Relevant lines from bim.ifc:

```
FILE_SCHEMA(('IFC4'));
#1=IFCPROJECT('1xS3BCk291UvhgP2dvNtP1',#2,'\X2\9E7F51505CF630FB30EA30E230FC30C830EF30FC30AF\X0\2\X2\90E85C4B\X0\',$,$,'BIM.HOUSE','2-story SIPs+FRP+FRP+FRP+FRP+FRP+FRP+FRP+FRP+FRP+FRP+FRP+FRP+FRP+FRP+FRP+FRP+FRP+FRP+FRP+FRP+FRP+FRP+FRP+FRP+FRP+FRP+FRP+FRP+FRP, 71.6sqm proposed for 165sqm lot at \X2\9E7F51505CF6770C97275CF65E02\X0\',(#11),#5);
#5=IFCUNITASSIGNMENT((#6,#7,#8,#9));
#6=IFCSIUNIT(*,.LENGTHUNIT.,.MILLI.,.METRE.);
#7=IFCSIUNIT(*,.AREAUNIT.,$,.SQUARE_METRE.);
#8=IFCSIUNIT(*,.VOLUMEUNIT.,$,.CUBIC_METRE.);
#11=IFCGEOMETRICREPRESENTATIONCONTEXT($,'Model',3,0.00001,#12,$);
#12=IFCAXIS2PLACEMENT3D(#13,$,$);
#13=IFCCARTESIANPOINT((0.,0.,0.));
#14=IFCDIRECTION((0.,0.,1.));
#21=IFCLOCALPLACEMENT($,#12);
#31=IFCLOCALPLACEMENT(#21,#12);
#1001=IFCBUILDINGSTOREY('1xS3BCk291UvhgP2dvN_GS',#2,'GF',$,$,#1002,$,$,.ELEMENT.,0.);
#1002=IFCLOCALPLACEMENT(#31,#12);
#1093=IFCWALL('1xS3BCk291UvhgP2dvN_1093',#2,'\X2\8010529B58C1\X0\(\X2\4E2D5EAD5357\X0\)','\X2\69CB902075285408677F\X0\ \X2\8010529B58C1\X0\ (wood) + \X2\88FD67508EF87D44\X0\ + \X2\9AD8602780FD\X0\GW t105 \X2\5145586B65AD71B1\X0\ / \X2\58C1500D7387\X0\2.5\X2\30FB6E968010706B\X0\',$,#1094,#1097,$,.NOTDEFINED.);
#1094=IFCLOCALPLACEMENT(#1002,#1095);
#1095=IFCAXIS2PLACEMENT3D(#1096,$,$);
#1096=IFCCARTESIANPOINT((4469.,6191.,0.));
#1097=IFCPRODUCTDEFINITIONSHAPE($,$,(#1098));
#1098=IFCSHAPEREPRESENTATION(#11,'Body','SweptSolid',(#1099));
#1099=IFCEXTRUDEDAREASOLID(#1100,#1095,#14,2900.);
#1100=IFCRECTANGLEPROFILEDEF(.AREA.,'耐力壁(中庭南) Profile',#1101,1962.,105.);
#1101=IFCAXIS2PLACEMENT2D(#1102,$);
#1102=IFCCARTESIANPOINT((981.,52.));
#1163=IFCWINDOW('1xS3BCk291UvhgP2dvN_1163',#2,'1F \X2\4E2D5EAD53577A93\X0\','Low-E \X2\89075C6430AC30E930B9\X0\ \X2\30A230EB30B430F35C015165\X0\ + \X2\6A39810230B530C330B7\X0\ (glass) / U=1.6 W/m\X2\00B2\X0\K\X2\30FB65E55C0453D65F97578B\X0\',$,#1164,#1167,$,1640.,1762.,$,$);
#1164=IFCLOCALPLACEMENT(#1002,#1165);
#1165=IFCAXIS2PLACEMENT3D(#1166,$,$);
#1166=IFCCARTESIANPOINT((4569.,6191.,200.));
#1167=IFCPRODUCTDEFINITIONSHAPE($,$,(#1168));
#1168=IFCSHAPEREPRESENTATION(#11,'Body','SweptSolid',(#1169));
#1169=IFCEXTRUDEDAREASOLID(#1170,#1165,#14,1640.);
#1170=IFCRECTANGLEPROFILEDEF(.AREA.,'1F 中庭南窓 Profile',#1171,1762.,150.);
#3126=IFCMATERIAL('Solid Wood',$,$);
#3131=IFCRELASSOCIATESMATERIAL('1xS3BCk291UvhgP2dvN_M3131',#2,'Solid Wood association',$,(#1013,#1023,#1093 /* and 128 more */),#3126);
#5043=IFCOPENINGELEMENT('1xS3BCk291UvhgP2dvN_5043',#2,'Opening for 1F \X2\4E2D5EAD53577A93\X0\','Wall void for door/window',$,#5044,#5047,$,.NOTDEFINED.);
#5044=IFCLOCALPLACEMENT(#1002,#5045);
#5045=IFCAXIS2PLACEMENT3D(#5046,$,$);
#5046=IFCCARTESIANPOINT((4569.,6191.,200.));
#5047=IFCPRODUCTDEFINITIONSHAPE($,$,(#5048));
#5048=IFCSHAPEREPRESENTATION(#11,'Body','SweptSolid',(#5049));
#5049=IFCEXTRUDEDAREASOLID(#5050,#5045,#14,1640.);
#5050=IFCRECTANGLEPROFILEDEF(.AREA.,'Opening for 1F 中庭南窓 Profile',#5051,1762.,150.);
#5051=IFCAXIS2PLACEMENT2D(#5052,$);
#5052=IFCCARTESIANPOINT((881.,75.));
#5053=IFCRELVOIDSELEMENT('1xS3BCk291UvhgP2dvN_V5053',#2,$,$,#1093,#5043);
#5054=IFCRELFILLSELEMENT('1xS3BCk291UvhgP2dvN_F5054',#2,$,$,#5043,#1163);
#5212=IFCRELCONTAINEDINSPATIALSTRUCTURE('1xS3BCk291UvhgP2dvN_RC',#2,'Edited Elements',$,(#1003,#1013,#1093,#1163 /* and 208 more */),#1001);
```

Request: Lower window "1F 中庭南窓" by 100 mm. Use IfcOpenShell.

```python
import numpy as np
import ifcopenshell
import ifcopenshell.api.geometry
import ifcopenshell.util.placement
import ifcopenshell.util.unit

model = ifcopenshell.open("bim.ifc")
unit_scale = ifcopenshell.util.unit.calculate_unit_scale(model)

window = model.by_guid("1xS3BCk291UvhgP2dvN_1163")
opening = window.FillsVoids[0].RelatingOpeningElement
dz = -100.0

shift = np.array([0.0, 0.0, dz])
# The window is not placed relative to its opening, so move both.
for product in (opening, window):
    matrix = ifcopenshell.util.placement.get_local_placement(product.ObjectPlacement)
    matrix[:3, 3] += shift
    ifcopenshell.api.geometry.edit_object_placement(model, product=product, matrix=matrix, is_si=False)

print(f"moved by {dz * unit_scale:+.3f} m")

model.write("bim-out.ifc")
```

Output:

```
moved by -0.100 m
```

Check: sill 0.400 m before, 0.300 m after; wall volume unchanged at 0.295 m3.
